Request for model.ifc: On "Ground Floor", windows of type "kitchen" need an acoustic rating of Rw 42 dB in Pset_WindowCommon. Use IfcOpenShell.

First a look at what the model holds.

```python
import ifcopenshell
import ifcopenshell.util.element

model = ifcopenshell.open("model.ifc")
print(model.schema)
storey = next(s for s in model.by_type("IfcBuildingStorey") if s.Name == "Ground Floor")
windows = [e for e in ifcopenshell.util.element.get_decomposition(storey) if e.is_a("IfcWindow")]
seen = {}
for e in windows:
    element_type = ifcopenshell.util.element.get_type(e)
    key = (element_type.Name if element_type != e and element_type else None, ifcopenshell.util.element.get_pset(e, "Pset_WindowCommon", "AcousticRating"))
    seen[key] = seen.get(key, 0) + 1
for (name, value), count in sorted(seen.items(), key=str):
    print(count, "x", name, "|", value)
```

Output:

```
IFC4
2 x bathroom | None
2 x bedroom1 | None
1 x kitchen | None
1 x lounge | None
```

```python
import ifcopenshell
import ifcopenshell.api.pset
import ifcopenshell.util.element

model = ifcopenshell.open("model.ifc")

storey = next(s for s in model.by_type("IfcBuildingStorey") if s.Name == "Ground Floor")
windows = [e for e in ifcopenshell.util.element.get_decomposition(storey) if e.is_a("IfcWindow")]

count = 0
for e in windows:
    element_type = ifcopenshell.util.element.get_type(e)
    if element_type in (None, e) or element_type.Name != "kitchen":
        continue
    # add_pset returns the element's existing set when there is one.
    pset = ifcopenshell.api.pset.add_pset(model, product=e, name="Pset_WindowCommon")
    ifcopenshell.api.pset.edit_pset(model, pset=pset, properties={"AcousticRating": "Rw 42 dB"})
    count += 1

print(count, "windows updated")

model.write("model_edited.ifc")
```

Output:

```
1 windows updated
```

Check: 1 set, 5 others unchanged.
